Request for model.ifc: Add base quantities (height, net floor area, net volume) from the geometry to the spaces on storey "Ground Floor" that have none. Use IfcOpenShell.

First a look at what the model holds.

```python
import ifcopenshell
import ifcopenshell.util.element
import ifcopenshell.util.unit

model = ifcopenshell.open("model.ifc")
print(model.schema)
for unit_type in ("LENGTHUNIT", "AREAUNIT", "VOLUMEUNIT"):
    print(unit_type, ifcopenshell.util.unit.calculate_unit_scale(model, unit_type))
storey = next(s for s in model.by_type("IfcBuildingStorey") if s.Name == "Ground Floor")
spaces = [e for e in ifcopenshell.util.element.get_decomposition(storey) if e.is_a("IfcSpace")]
for e in sorted(spaces, key=lambda e: e.id()):
    print(e.id(), e.is_a(), e.Name, list(ifcopenshell.util.element.get_psets(e, qtos_only=True)), sep=" | ")
```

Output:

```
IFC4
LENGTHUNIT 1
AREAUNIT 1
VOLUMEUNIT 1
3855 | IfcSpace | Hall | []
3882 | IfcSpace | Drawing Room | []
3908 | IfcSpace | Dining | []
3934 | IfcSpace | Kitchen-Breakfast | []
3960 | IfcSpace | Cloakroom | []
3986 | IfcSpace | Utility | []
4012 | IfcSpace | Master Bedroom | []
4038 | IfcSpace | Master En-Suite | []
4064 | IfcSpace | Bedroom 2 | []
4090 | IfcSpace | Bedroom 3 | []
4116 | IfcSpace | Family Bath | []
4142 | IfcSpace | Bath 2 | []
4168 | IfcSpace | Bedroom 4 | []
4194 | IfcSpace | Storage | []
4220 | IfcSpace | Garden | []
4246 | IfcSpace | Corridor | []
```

```python
import ifcopenshell
import ifcopenshell.api.pset
import ifcopenshell.geom
import ifcopenshell.util.element
import ifcopenshell.util.shape
import ifcopenshell.util.unit

model = ifcopenshell.open("model.ifc")
unit_scale = ifcopenshell.util.unit.calculate_unit_scale(model)
area_scale = ifcopenshell.util.unit.calculate_unit_scale(model, "AREAUNIT")
volume_scale = ifcopenshell.util.unit.calculate_unit_scale(model, "VOLUMEUNIT")
settings = ifcopenshell.geom.settings()

storey = next(s for s in model.by_type("IfcBuildingStorey") if s.Name == "Ground Floor")
spaces = [e for e in ifcopenshell.util.element.get_decomposition(storey) if e.is_a("IfcSpace")]

for e in sorted(spaces, key=lambda e: e.id()):
    if ifcopenshell.util.element.get_psets(e, qtos_only=True, should_inherit=False):
        continue
    # Geometry comes back in metres, in the element's own axes.
    shape = ifcopenshell.geom.create_shape(settings, e)
    values = {
        "Height": ifcopenshell.util.shape.get_z(shape.geometry) / unit_scale,
        "NetFloorArea": ifcopenshell.util.shape.get_footprint_area(shape.geometry) / area_scale,
        "NetVolume": ifcopenshell.util.shape.get_volume(shape.geometry) / volume_scale,
    }
    qto = ifcopenshell.api.pset.add_qto(model, product=e, name="Qto_SpaceBaseQuantities")
    ifcopenshell.api.pset.edit_qto(model, qto=qto, properties=values)
    print(e.id(), {k: round(v, 3) for k, v in values.items()})

model.write("model_rev.ifc")
```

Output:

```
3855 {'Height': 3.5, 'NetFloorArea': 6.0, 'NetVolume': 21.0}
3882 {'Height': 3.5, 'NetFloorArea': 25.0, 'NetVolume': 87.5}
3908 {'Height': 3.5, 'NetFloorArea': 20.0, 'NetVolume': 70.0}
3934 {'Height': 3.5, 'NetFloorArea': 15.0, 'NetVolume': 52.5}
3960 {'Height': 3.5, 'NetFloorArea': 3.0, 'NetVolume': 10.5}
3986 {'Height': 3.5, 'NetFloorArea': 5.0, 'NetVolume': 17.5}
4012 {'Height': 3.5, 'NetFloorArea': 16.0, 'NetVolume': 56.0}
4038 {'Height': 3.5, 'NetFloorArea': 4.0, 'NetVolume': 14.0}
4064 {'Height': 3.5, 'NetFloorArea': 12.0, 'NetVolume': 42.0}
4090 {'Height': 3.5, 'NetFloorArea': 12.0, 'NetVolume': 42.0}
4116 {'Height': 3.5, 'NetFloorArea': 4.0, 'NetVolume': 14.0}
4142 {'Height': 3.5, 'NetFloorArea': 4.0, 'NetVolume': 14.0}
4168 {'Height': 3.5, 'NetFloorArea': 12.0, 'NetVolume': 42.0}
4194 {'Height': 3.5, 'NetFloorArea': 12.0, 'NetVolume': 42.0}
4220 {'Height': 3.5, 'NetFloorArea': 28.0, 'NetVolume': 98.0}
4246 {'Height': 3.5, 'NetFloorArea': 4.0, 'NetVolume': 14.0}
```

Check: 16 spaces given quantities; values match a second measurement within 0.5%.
